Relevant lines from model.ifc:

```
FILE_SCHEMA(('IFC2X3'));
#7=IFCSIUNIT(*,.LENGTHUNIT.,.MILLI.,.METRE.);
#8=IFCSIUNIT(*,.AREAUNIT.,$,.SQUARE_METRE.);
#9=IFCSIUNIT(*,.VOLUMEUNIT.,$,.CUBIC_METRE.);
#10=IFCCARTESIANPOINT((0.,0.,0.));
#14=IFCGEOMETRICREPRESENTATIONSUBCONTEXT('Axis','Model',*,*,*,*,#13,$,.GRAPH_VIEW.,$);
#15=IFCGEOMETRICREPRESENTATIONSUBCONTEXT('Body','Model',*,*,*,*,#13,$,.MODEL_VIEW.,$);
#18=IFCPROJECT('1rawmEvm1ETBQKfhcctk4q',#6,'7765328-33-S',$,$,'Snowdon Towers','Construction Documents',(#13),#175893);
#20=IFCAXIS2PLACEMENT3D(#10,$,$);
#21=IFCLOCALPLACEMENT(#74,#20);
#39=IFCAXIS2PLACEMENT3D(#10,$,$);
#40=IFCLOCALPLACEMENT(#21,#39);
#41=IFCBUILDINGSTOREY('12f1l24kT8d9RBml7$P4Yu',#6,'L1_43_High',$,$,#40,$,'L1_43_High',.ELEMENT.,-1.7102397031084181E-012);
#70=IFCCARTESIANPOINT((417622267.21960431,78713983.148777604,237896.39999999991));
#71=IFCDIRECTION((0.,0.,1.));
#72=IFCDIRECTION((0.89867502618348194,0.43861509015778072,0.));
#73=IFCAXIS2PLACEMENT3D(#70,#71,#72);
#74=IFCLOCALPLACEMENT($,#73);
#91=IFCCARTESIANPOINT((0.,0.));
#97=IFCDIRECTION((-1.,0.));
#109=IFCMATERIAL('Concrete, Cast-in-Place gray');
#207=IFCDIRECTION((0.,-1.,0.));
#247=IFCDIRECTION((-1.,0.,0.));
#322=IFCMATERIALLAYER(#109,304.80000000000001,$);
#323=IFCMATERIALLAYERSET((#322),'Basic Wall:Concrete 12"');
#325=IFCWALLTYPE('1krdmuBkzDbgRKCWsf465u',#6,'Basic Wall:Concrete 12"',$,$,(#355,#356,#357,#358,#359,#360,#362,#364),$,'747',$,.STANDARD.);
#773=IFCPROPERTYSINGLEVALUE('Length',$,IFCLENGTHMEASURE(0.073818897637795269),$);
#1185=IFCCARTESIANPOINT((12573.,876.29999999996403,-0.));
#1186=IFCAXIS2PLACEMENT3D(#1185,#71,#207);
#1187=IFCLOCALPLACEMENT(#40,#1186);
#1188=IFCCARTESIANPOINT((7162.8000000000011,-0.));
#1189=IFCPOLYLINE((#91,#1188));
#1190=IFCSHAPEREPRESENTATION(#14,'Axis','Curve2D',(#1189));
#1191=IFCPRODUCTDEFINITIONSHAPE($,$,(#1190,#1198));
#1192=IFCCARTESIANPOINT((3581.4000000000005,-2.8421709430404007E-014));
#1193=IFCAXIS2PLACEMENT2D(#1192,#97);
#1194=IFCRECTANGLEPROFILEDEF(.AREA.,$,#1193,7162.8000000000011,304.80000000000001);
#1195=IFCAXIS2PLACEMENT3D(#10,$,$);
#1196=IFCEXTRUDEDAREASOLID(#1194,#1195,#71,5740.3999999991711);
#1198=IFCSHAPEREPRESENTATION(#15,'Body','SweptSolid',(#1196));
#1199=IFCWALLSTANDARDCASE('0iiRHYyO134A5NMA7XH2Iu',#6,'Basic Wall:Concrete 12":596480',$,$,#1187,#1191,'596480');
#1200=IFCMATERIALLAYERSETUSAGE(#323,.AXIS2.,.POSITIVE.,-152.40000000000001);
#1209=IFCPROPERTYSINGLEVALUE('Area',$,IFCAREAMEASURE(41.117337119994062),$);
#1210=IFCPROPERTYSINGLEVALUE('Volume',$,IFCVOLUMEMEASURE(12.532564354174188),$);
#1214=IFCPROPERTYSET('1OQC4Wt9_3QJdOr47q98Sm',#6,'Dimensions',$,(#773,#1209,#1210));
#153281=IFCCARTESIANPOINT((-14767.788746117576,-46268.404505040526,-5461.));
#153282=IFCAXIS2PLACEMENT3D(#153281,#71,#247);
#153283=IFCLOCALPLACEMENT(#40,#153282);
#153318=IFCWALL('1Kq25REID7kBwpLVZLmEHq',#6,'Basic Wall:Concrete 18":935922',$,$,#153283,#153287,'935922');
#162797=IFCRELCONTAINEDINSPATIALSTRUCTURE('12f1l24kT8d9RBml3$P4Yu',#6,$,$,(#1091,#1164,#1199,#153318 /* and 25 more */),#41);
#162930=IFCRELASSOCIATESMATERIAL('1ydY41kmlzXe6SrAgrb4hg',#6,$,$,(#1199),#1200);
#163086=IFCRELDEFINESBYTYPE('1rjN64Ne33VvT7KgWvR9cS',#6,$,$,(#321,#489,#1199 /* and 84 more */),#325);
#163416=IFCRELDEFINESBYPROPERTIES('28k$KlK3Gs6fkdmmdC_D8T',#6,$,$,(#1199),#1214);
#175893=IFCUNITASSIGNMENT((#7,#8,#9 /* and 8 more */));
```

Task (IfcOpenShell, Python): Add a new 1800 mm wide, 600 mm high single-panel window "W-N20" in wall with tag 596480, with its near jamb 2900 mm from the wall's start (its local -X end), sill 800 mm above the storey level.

```python
import numpy as np
import ifcopenshell
import ifcopenshell.api.feature
import ifcopenshell.api.geometry
import ifcopenshell.api.pset
import ifcopenshell.api.root
import ifcopenshell.api.spatial
import ifcopenshell.api.type
import ifcopenshell.geom
import ifcopenshell.util.element
import ifcopenshell.util.placement
import ifcopenshell.util.representation
import ifcopenshell.util.shape
import ifcopenshell.util.unit

model = ifcopenshell.open("model.ifc")
unit_scale = ifcopenshell.util.unit.calculate_unit_scale(model)
area_scale = ifcopenshell.util.unit.calculate_unit_scale(model, "AREAUNIT")
volume_scale = ifcopenshell.util.unit.calculate_unit_scale(model, "VOLUMEUNIT")
settings = ifcopenshell.geom.settings()


def volume(element):
    """Net volume in cubic metres, openings subtracted."""
    shape = ifcopenshell.geom.create_shape(settings, element)
    return ifcopenshell.util.shape.get_volume(shape.geometry)


wall = model.by_guid("0iiRHYyO134A5NMA7XH2Iu")
storey = ifcopenshell.util.element.get_container(wall, ifc_class="IfcBuildingStorey")
context = ifcopenshell.util.representation.get_context(model, "Model", "Body", "MODEL_VIEW")
before = volume(wall)

width, height, from_end, sill = 1.8, 0.6, 2.9, 0.8  # metres

# The wall runs along its own X axis, and the end named is its -X end.
wall_shape = ifcopenshell.geom.create_shape(settings, wall)
x, y, z = ifcopenshell.util.shape.get_vertices(wall_shape.geometry).T
start = x.min() + from_end
face, thickness = float(y.min()), float(y.max() - y.min())
wall_matrix = ifcopenshell.util.placement.get_local_placement(wall.ObjectPlacement)
level = ifcopenshell.util.placement.get_local_placement(storey.ObjectPlacement)[2, 3]


def in_wall(x, y):
    """Placement at x, y metres in the wall's axes, at sill height."""
    matrix = wall_matrix.copy()
    matrix[:, 3] = wall_matrix @ np.array([x / unit_scale, y / unit_scale, 0.0, 1.0])
    matrix[2, 3] = level + sill / unit_scale
    return matrix


# Opening: a box that overshoots both wall faces by 50 mm.
opening = ifcopenshell.api.root.create_entity(model, ifc_class="IfcOpeningElement")
box = ifcopenshell.api.geometry.add_wall_representation(
    model, context=context, length=width, height=height, thickness=thickness + 0.1
)
ifcopenshell.api.geometry.assign_representation(model, product=opening, representation=box)
ifcopenshell.api.geometry.edit_object_placement(model, product=opening, matrix=in_wall(start, face - 0.05), is_si=False)
ifcopenshell.api.feature.add_feature(model, feature=opening, element=wall)

window = ifcopenshell.api.root.create_entity(model, ifc_class="IfcWindow", name="W-N20")
window.OverallWidth, window.OverallHeight = width / unit_scale, height / unit_scale
body = ifcopenshell.api.geometry.add_window_representation(
    model,
    context=context,
    overall_width=window.OverallWidth,
    overall_height=window.OverallHeight,
    partition_type="SINGLE_PANEL",
)
ifcopenshell.api.geometry.assign_representation(model, product=window, representation=body)
ifcopenshell.api.spatial.assign_container(model, products=[window], relating_structure=storey)
fills = ifcopenshell.api.feature.add_filling(model, opening=opening, element=window)
fills.OwnerHistory = window.OwnerHistory  # required in IFC2X3

# IFC2X3 keeps the operation on the window style.
style = ifcopenshell.api.root.create_entity(model, ifc_class="IfcWindowStyle", name="W-N20")
style.OperationType, style.ConstructionType = "SINGLE_PANEL", "NOTDEFINED"
style.ParameterTakesPrecedence = style.Sizeable = False
ifcopenshell.api.type.assign_type(model, related_objects=[window], relating_type=style)

# Centre the window in the wall's thickness.
ifcopenshell.api.geometry.edit_object_placement(model, product=window, matrix=in_wall(start, face), is_si=False)
window_shape = ifcopenshell.geom.create_shape(settings, window)
depth = ifcopenshell.util.shape.get_vertices(window_shape.geometry)[:, 1]
offset = face + thickness / 2 - (depth.min() + depth.max()) / 2
ifcopenshell.api.geometry.edit_object_placement(model, product=window, matrix=in_wall(start, offset), is_si=False)

after = volume(wall)

# Update the wall's stored quantities.
pset = model.by_id(ifcopenshell.util.element.get_pset(wall, "Dimensions", should_inherit=False)["id"])
ifcopenshell.api.pset.edit_pset(model, pset=pset, properties={
    "Area": model.create_entity("IfcAreaMeasure", after / thickness / area_scale),
    "Volume": model.create_entity("IfcVolumeMeasure", after / volume_scale),
})

print(f"wall volume {before:.3f} -> {after:.3f} m3")

model.write("model_rev.ifc")
```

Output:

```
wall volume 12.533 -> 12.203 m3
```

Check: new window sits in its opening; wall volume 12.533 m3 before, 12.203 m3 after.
